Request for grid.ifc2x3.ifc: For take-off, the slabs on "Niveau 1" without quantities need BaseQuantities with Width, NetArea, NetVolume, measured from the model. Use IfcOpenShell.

First a look at what the model holds.

```python
import ifcopenshell
import ifcopenshell.util.element
import ifcopenshell.util.unit

model = ifcopenshell.open("grid.ifc2x3.ifc")
print(model.schema)
for unit_type in ("LENGTHUNIT", "AREAUNIT", "VOLUMEUNIT"):
    print(unit_type, ifcopenshell.util.unit.calculate_unit_scale(model, unit_type))
storey = next(s for s in model.by_type("IfcBuildingStorey") if s.Name == "Niveau 1")
slabs = [e for e in ifcopenshell.util.element.get_decomposition(storey) if e.is_a("IfcSlab")]
for e in sorted(slabs, key=lambda e: e.id()):
    print(e.id(), e.is_a(), e.Name, list(ifcopenshell.util.element.get_psets(e, qtos_only=True)), sep=" | ")
```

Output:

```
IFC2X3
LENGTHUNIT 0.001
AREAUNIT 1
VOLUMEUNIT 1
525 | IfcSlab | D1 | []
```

```python
import ifcopenshell
import ifcopenshell.api.pset
import ifcopenshell.geom
import ifcopenshell.util.element
import ifcopenshell.util.shape
import ifcopenshell.util.unit

model = ifcopenshell.open("grid.ifc2x3.ifc")
unit_scale = ifcopenshell.util.unit.calculate_unit_scale(model)
area_scale = ifcopenshell.util.unit.calculate_unit_scale(model, "AREAUNIT")
volume_scale = ifcopenshell.util.unit.calculate_unit_scale(model, "VOLUMEUNIT")
settings = ifcopenshell.geom.settings()

storey = next(s for s in model.by_type("IfcBuildingStorey") if s.Name == "Niveau 1")
slabs = [e for e in ifcopenshell.util.element.get_decomposition(storey) if e.is_a("IfcSlab")]

for e in sorted(slabs, key=lambda e: e.id()):
    if ifcopenshell.util.element.get_psets(e, qtos_only=True, should_inherit=False):
        continue
    # Geometry comes back in metres, in the element's own axes.
    shape = ifcopenshell.geom.create_shape(settings, e)
    values = {
        "Width": ifcopenshell.util.shape.get_z(shape.geometry) / unit_scale,
        "NetArea": ifcopenshell.util.shape.get_footprint_area(shape.geometry) / area_scale,
        "NetVolume": ifcopenshell.util.shape.get_volume(shape.geometry) / volume_scale,
    }
    qto = ifcopenshell.api.pset.add_qto(model, product=e, name="BaseQuantities")
    ifcopenshell.api.pset.edit_qto(model, qto=qto, properties=values)
    print(e.id(), {k: round(v, 3) for k, v in values.items()})

model.write("grid.ifc2x3_edited.ifc")
```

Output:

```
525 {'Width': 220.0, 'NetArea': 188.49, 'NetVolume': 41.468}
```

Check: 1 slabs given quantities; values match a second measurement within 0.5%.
